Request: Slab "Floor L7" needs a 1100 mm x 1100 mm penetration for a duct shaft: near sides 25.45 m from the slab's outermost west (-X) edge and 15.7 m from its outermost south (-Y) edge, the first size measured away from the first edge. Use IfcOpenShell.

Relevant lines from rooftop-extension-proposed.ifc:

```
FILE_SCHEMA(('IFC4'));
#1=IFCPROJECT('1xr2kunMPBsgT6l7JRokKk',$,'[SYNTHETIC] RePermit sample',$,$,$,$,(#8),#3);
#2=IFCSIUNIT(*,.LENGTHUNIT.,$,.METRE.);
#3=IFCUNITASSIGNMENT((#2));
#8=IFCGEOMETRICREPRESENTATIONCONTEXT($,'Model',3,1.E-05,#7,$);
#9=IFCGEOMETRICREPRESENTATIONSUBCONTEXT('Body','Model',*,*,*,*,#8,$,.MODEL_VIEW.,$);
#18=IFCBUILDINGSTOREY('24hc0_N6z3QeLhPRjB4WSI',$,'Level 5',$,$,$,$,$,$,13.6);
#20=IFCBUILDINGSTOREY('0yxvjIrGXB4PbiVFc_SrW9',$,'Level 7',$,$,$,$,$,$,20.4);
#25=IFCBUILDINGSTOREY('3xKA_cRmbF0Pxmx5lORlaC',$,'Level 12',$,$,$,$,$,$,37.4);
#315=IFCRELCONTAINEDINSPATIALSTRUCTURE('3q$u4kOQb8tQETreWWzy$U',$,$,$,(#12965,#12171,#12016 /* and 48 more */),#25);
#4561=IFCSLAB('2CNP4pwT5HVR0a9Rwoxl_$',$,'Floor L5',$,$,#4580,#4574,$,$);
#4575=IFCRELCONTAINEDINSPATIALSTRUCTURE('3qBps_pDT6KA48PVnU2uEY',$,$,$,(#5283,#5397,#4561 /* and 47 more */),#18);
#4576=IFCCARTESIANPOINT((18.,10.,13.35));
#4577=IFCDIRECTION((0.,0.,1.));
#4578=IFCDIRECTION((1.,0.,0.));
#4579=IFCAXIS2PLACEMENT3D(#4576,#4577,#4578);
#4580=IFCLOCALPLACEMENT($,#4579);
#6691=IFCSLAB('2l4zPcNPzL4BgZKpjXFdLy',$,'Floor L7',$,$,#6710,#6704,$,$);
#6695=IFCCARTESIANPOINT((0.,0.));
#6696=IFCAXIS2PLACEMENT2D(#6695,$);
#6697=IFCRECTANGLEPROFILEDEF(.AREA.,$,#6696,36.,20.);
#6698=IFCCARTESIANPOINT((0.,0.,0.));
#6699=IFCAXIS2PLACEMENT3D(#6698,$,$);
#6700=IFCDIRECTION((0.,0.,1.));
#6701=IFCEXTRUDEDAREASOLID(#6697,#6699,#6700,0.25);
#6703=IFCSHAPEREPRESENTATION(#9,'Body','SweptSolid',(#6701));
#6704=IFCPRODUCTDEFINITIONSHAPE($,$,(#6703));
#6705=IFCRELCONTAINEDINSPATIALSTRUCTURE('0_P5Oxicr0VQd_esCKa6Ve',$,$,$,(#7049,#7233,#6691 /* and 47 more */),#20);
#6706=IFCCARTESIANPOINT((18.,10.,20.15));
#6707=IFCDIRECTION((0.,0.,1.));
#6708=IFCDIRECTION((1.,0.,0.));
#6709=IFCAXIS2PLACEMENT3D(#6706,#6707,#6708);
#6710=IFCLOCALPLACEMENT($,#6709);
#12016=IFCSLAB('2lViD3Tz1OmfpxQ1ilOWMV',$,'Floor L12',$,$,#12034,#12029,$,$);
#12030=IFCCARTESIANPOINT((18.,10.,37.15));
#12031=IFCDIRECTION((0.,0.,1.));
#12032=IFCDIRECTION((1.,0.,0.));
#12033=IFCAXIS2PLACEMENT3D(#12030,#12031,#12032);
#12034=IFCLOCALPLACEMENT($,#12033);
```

```python
import numpy as np
import ifcopenshell
import ifcopenshell.api.feature
import ifcopenshell.api.geometry
import ifcopenshell.api.root
import ifcopenshell.geom
import ifcopenshell.util.placement
import ifcopenshell.util.representation
import ifcopenshell.util.shape
import ifcopenshell.util.unit

model = ifcopenshell.open("rooftop-extension-proposed.ifc")
unit_scale = ifcopenshell.util.unit.calculate_unit_scale(model)
settings = ifcopenshell.geom.settings()


def volume(element):
    """Net volume in cubic metres, openings subtracted."""
    shape = ifcopenshell.geom.create_shape(settings, element)
    return ifcopenshell.util.shape.get_volume(shape.geometry)


slab = model.by_guid("2l4zPcNPzL4BgZKpjXFdLy")
before = volume(slab)

# Extent in the slab's own axes, in metres. The edges named are its -X and -Y sides.
slab_shape = ifcopenshell.geom.create_shape(settings, slab)
vertices = ifcopenshell.util.shape.get_vertices(slab_shape.geometry)
x_min, y_min, bottom = vertices.min(axis=0)
top = vertices[:, 2].max()

opening = ifcopenshell.api.root.create_entity(model, ifc_class="IfcOpeningElement", name="Duct shaft opening", predefined_type="OPENING")
context = ifcopenshell.util.representation.get_context(model, "Model", "Body", "MODEL_VIEW")
width, depth = 1.1, 1.1
outline = [(0.0, 0.0), (width, 0.0), (width, depth), (0.0, depth), (0.0, 0.0)]
# Overshoot both faces by 50 mm so the cut is clean.
shape = ifcopenshell.api.geometry.add_slab_representation(
    model, context=context, depth=top - bottom + 0.1, polyline=outline
)
ifcopenshell.api.geometry.assign_representation(model, product=opening, representation=shape)

matrix = ifcopenshell.util.placement.get_local_placement(slab.ObjectPlacement)
matrix[:, 3] = matrix @ np.append(np.array([x_min + 25.45, y_min + 15.7, bottom - 0.05]) / unit_scale, 1.0)
ifcopenshell.api.geometry.edit_object_placement(model, product=opening, matrix=matrix, is_si=False)
ifcopenshell.api.feature.add_feature(model, feature=opening, element=slab)

after = volume(slab)

print(f"slab volume {before:.3f} -> {after:.3f} m3")

model.write("rooftop-extension-proposed_v2.ifc")
```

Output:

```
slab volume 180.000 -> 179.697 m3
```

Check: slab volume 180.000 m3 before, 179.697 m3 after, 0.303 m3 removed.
